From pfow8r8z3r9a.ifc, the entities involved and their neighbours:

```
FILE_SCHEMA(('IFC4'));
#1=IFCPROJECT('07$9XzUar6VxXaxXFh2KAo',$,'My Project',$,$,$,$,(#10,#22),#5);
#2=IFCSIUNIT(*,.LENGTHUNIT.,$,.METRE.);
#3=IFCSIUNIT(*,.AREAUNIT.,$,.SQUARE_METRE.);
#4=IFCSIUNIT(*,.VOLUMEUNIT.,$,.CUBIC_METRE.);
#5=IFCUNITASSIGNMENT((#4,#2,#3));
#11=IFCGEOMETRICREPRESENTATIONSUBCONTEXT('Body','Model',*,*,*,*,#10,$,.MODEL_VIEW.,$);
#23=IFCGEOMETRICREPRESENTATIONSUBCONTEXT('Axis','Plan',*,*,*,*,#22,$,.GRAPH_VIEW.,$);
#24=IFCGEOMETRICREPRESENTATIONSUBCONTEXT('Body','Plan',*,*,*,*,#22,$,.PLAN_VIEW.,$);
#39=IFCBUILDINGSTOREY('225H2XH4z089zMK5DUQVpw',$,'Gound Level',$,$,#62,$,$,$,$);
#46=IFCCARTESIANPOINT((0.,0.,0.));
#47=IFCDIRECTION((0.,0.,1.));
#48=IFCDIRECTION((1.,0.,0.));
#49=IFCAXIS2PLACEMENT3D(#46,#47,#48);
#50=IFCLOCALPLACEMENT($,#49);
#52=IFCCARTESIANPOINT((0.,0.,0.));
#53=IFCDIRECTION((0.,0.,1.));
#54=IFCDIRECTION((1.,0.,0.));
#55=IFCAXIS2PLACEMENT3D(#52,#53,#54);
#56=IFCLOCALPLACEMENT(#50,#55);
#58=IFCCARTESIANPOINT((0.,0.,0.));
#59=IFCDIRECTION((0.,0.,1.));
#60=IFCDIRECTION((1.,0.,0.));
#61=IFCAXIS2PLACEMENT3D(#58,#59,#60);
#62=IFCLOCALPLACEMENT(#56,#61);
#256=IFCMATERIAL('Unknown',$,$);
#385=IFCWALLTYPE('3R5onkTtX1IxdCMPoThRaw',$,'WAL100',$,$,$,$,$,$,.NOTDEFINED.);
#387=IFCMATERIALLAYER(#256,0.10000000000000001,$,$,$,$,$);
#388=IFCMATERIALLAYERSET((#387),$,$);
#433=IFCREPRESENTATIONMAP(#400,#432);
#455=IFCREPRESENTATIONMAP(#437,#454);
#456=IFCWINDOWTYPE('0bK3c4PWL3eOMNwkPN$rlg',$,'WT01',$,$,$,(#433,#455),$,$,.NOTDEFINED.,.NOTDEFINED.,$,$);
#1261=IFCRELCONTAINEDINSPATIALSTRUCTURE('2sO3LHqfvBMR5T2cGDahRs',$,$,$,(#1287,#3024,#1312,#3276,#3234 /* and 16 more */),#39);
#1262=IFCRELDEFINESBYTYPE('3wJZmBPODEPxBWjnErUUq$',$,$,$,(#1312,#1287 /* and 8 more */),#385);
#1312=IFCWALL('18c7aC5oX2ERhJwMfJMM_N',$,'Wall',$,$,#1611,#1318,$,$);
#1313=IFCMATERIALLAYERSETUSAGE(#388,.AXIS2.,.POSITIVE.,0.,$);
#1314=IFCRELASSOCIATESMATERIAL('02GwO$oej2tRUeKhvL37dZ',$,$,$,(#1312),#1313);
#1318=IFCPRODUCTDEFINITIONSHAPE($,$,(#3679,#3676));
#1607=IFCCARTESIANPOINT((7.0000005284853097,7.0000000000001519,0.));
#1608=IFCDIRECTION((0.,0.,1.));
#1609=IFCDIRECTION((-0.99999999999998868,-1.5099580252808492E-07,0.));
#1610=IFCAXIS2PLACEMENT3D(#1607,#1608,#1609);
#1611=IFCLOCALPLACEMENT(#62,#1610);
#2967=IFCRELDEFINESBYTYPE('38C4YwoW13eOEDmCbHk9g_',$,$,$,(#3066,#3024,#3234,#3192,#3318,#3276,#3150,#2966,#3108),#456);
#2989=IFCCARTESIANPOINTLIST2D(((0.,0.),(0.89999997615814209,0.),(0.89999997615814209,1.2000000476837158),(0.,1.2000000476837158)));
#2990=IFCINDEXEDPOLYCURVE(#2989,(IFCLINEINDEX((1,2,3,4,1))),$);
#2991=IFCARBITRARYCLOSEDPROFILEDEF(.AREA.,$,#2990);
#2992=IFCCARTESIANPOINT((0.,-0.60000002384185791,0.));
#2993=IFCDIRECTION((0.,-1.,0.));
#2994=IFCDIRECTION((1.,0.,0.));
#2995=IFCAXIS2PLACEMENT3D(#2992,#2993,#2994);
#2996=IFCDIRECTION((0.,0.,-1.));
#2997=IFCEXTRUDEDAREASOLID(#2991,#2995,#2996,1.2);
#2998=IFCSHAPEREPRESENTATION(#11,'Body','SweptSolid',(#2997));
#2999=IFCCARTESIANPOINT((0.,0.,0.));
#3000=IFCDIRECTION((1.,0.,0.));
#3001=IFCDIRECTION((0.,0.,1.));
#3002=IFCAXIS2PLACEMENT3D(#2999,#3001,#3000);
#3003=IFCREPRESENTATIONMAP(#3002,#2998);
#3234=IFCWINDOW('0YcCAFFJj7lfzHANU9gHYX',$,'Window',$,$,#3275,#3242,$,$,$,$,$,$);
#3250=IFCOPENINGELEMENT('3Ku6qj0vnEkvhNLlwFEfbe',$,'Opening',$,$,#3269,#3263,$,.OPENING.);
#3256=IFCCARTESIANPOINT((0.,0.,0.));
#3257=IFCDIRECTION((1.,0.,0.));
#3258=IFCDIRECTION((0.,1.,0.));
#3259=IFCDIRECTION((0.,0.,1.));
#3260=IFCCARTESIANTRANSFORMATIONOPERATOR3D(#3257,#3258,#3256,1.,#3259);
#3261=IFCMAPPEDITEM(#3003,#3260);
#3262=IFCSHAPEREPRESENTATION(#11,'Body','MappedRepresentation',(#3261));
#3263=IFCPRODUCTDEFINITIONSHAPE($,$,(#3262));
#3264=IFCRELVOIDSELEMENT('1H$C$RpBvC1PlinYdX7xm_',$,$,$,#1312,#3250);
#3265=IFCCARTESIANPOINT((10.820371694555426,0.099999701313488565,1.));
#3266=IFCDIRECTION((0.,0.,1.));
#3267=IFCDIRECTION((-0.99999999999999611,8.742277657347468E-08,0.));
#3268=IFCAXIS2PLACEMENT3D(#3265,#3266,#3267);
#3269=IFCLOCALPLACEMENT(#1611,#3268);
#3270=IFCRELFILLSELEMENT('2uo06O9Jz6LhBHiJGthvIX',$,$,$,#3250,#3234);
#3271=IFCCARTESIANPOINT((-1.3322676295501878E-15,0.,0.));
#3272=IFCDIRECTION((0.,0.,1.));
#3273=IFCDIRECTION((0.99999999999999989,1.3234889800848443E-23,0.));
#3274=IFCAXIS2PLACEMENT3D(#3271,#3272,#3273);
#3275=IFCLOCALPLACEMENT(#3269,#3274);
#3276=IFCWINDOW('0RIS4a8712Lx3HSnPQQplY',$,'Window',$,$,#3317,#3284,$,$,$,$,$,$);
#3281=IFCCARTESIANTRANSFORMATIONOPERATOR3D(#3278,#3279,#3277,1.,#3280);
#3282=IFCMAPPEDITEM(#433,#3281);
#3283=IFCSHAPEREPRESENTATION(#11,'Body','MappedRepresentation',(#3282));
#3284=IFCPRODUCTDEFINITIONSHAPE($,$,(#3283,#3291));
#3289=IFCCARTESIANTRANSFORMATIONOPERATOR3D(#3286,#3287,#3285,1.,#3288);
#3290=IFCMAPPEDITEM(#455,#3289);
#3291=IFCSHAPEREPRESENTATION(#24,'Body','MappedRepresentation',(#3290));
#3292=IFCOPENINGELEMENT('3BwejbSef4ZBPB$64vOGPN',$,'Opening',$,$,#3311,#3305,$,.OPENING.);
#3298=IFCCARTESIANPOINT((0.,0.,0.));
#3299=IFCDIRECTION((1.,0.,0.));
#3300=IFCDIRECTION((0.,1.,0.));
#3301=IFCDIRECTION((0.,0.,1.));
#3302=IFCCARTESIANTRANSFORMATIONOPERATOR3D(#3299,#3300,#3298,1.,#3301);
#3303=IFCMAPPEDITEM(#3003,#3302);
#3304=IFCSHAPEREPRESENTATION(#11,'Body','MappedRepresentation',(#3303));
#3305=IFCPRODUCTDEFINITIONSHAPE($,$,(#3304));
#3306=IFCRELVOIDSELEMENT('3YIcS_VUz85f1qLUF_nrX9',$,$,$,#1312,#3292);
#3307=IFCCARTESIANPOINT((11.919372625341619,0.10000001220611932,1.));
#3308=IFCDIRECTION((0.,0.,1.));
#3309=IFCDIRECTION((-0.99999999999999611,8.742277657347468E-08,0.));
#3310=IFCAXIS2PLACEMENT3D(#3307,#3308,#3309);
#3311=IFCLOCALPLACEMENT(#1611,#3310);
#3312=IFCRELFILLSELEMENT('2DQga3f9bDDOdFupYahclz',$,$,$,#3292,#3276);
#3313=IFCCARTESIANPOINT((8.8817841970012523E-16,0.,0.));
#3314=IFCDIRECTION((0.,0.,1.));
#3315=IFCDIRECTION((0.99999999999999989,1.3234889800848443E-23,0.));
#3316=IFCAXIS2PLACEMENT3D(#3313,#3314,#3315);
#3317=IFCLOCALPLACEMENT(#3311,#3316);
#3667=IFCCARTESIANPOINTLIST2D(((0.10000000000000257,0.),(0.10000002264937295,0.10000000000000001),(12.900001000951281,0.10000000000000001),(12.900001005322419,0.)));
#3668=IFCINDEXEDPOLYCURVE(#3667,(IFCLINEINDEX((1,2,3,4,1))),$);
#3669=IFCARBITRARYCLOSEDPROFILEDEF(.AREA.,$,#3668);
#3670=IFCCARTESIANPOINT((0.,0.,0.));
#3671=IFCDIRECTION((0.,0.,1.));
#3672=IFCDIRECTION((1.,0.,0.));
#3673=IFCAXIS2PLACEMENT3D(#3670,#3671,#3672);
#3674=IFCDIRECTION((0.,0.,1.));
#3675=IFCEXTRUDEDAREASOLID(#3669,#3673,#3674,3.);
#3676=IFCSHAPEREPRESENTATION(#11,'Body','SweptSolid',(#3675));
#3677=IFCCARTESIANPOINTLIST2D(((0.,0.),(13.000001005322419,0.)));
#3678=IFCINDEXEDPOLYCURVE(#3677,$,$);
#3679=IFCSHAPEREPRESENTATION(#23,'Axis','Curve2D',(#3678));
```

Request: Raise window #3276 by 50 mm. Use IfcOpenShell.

```python
import numpy as np
import ifcopenshell
import ifcopenshell.api.geometry
import ifcopenshell.util.placement
import ifcopenshell.util.unit

model = ifcopenshell.open("pfow8r8z3r9a.ifc")
unit_scale = ifcopenshell.util.unit.calculate_unit_scale(model)

window = model.by_guid("0RIS4a8712Lx3HSnPQQplY")
opening = window.FillsVoids[0].RelatingOpeningElement
dz = 0.05 / unit_scale

shift = np.array([0.0, 0.0, dz])
# The window is placed relative to its opening, so it follows when the opening moves.
matrix = ifcopenshell.util.placement.get_local_placement(opening.ObjectPlacement)
matrix[:3, 3] += shift
ifcopenshell.api.geometry.edit_object_placement(
    model, product=opening, matrix=matrix, is_si=False, should_transform_children=True
)

print(f"moved by {dz * unit_scale:+.3f} m")

model.write("pfow8r8z3r9a_v2.ifc")
```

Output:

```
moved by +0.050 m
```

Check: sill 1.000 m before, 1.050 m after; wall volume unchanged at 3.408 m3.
